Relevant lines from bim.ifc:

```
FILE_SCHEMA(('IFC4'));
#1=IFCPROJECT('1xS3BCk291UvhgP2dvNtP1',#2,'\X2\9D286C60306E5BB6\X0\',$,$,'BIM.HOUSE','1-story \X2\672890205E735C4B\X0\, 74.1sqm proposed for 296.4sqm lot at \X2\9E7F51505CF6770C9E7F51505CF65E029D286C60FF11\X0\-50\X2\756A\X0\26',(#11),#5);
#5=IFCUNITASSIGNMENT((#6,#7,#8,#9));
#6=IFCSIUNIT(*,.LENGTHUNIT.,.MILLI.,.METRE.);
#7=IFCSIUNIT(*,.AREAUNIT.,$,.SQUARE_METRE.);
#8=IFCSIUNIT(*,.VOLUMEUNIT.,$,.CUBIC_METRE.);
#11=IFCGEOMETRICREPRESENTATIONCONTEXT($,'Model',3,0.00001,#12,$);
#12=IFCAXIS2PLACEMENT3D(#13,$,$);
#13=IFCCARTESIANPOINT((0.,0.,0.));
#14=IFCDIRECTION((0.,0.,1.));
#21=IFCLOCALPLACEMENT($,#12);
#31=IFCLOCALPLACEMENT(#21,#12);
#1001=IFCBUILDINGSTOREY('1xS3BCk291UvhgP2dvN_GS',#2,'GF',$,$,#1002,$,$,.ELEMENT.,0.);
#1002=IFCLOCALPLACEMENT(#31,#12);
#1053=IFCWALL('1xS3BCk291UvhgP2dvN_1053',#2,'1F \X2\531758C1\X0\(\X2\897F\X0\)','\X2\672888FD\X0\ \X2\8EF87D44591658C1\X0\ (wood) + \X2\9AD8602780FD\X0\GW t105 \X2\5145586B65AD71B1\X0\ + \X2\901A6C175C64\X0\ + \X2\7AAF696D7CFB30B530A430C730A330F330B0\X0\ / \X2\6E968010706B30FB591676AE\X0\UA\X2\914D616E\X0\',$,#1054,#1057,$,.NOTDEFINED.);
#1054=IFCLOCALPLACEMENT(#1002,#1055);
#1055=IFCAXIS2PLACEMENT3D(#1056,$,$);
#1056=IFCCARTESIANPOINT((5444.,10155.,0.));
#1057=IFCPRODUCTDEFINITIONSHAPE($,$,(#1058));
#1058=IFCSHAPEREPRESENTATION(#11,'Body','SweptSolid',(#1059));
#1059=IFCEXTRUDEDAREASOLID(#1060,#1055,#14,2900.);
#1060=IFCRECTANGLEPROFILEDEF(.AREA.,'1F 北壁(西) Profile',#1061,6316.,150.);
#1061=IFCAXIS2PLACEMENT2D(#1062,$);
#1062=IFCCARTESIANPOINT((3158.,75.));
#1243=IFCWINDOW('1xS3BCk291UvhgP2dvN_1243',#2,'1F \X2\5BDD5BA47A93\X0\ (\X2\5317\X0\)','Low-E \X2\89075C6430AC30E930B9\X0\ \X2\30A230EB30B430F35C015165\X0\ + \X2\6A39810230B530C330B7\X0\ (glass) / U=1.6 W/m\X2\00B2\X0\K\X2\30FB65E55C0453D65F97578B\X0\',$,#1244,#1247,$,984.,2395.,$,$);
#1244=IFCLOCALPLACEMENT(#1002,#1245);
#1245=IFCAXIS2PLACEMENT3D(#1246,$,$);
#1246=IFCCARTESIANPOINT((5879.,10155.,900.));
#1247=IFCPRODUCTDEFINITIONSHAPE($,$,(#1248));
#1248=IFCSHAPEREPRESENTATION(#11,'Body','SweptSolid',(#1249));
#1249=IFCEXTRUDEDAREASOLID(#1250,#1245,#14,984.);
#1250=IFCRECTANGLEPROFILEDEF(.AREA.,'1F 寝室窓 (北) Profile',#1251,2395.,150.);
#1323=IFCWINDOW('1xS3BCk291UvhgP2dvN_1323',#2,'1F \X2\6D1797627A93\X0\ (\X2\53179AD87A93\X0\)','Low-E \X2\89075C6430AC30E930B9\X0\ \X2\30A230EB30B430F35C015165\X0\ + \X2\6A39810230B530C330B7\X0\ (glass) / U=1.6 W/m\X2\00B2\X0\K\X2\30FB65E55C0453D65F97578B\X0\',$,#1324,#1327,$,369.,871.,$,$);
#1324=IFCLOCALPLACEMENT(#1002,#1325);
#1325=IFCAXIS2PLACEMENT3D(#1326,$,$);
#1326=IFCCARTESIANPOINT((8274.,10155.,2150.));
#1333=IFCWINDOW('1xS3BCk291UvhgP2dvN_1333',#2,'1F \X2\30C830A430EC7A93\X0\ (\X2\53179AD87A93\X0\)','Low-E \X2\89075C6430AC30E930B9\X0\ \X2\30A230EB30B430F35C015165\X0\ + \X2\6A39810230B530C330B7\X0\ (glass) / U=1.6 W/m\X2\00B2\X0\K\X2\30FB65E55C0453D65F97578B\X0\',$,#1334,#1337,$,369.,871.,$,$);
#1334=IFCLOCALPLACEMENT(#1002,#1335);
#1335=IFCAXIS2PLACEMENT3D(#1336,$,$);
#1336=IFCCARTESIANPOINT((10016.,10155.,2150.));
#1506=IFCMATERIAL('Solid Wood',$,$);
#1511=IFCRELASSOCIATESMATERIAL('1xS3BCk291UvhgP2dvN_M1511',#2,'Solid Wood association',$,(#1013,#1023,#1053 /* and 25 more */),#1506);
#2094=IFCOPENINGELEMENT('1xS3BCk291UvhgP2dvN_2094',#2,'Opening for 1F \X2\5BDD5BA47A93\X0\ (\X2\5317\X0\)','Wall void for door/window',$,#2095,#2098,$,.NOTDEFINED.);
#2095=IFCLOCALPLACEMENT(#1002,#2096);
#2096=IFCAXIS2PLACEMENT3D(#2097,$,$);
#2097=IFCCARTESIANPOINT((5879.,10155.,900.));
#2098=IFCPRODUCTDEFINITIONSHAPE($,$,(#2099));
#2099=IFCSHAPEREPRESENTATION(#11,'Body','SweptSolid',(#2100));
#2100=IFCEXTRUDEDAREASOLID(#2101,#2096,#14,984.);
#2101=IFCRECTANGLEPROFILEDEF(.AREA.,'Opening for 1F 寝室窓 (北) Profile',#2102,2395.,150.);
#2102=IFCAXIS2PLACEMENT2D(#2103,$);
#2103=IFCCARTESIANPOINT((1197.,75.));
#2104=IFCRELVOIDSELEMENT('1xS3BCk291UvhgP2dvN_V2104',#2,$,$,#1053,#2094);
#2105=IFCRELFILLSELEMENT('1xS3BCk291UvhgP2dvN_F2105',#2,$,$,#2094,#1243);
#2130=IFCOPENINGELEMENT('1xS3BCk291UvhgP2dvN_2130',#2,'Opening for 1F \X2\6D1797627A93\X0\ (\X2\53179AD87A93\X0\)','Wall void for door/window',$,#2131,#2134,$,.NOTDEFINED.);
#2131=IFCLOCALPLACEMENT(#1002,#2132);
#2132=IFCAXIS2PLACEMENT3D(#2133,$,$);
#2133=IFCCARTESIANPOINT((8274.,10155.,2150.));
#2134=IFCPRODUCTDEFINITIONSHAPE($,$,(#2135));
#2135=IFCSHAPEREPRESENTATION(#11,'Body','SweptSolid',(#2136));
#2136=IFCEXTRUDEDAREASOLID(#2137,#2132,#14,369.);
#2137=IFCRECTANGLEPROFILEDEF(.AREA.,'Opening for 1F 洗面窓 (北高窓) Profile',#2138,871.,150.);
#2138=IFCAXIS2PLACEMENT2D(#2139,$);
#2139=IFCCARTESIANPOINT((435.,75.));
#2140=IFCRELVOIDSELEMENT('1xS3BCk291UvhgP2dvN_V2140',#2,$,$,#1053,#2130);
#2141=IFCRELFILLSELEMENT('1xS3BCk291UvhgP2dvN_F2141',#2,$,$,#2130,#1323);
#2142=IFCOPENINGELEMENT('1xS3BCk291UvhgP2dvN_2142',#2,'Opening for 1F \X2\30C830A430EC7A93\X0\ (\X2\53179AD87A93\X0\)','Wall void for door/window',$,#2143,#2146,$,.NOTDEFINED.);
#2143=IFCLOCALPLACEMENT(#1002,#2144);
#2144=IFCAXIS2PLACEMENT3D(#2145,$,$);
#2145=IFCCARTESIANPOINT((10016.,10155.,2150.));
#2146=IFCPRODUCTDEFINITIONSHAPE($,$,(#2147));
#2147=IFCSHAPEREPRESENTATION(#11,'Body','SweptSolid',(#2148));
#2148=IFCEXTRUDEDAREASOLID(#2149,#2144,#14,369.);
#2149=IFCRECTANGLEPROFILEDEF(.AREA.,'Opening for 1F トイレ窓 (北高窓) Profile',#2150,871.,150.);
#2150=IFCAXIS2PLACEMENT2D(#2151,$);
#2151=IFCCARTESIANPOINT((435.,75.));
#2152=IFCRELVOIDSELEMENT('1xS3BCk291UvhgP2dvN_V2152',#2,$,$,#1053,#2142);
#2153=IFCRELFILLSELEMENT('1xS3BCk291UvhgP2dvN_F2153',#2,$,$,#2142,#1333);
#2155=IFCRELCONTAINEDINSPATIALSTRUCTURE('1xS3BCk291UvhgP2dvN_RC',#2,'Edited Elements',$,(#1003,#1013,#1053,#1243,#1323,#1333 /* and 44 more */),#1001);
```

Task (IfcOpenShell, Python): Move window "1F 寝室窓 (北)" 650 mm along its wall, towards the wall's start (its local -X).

```python
import ifcopenshell
import ifcopenshell.api.geometry
import ifcopenshell.util.placement
import ifcopenshell.util.unit

model = ifcopenshell.open("bim.ifc")
unit_scale = ifcopenshell.util.unit.calculate_unit_scale(model)

window = model.by_id(1243)
opening = window.FillsVoids[0].RelatingOpeningElement
wall = opening.VoidsElements[0].RelatingBuildingElement

wall_matrix = ifcopenshell.util.placement.get_local_placement(wall.ObjectPlacement)
shift = wall_matrix[:3, 0] * -0.65 / unit_scale
before = ifcopenshell.util.placement.get_local_placement(window.ObjectPlacement)[:3, 3].copy()

# The window is not placed relative to its opening, so move both.
for product in (opening, window):
    matrix = ifcopenshell.util.placement.get_local_placement(product.ObjectPlacement)
    matrix[:3, 3] += shift
    ifcopenshell.api.geometry.edit_object_placement(model, product=product, matrix=matrix, is_si=False)

after = ifcopenshell.util.placement.get_local_placement(window.ObjectPlacement)[:3, 3]
print("window moved by", (after - before).round(3) + 0.0)

model.write("bim_v2.ifc")
```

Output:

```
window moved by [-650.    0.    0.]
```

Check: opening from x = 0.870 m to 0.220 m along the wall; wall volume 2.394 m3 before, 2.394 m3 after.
